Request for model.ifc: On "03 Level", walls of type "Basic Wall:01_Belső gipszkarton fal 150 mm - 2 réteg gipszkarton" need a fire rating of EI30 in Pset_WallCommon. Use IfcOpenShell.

First a look at what the model holds.

```python
import ifcopenshell
import ifcopenshell.util.element

model = ifcopenshell.open("model.ifc")
print(model.schema)
storey = next(s for s in model.by_type("IfcBuildingStorey") if s.Name == "03 Level")
walls = [e for e in ifcopenshell.util.element.get_decomposition(storey) if e.is_a("IfcWall")]
seen = {}
for e in walls:
    element_type = ifcopenshell.util.element.get_type(e)
    key = (element_type.Name if element_type != e and element_type else None, ifcopenshell.util.element.get_pset(e, "Pset_WallCommon", "FireRating"))
    seen[key] = seen.get(key, 0) + 1
for (name, value), count in sorted(seen.items(), key=str):
    print(count, "x", name, "|", value)
```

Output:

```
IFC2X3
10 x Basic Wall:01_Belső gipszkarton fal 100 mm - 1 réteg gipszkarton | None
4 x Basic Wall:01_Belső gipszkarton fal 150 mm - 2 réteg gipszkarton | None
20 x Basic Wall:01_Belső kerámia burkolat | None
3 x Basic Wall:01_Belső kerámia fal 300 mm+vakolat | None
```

```python
import ifcopenshell
import ifcopenshell.api.pset
import ifcopenshell.util.element

model = ifcopenshell.open("model.ifc")

storey = next(s for s in model.by_type("IfcBuildingStorey") if s.Name == "03 Level")
walls = [e for e in ifcopenshell.util.element.get_decomposition(storey) if e.is_a("IfcWall")]

count = 0
for e in walls:
    element_type = ifcopenshell.util.element.get_type(e)
    if element_type in (None, e) or element_type.Name != "Basic Wall:01_Belső gipszkarton fal 150 mm - 2 réteg gipszkarton":
        continue
    # add_pset returns the element's existing set when there is one.
    pset = ifcopenshell.api.pset.add_pset(model, product=e, name="Pset_WallCommon")
    ifcopenshell.api.pset.edit_pset(model, pset=pset, properties={"FireRating": "EI30"})
    count += 1

print(count, "walls updated")

model.write("model-out.ifc")
```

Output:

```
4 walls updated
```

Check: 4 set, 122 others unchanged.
